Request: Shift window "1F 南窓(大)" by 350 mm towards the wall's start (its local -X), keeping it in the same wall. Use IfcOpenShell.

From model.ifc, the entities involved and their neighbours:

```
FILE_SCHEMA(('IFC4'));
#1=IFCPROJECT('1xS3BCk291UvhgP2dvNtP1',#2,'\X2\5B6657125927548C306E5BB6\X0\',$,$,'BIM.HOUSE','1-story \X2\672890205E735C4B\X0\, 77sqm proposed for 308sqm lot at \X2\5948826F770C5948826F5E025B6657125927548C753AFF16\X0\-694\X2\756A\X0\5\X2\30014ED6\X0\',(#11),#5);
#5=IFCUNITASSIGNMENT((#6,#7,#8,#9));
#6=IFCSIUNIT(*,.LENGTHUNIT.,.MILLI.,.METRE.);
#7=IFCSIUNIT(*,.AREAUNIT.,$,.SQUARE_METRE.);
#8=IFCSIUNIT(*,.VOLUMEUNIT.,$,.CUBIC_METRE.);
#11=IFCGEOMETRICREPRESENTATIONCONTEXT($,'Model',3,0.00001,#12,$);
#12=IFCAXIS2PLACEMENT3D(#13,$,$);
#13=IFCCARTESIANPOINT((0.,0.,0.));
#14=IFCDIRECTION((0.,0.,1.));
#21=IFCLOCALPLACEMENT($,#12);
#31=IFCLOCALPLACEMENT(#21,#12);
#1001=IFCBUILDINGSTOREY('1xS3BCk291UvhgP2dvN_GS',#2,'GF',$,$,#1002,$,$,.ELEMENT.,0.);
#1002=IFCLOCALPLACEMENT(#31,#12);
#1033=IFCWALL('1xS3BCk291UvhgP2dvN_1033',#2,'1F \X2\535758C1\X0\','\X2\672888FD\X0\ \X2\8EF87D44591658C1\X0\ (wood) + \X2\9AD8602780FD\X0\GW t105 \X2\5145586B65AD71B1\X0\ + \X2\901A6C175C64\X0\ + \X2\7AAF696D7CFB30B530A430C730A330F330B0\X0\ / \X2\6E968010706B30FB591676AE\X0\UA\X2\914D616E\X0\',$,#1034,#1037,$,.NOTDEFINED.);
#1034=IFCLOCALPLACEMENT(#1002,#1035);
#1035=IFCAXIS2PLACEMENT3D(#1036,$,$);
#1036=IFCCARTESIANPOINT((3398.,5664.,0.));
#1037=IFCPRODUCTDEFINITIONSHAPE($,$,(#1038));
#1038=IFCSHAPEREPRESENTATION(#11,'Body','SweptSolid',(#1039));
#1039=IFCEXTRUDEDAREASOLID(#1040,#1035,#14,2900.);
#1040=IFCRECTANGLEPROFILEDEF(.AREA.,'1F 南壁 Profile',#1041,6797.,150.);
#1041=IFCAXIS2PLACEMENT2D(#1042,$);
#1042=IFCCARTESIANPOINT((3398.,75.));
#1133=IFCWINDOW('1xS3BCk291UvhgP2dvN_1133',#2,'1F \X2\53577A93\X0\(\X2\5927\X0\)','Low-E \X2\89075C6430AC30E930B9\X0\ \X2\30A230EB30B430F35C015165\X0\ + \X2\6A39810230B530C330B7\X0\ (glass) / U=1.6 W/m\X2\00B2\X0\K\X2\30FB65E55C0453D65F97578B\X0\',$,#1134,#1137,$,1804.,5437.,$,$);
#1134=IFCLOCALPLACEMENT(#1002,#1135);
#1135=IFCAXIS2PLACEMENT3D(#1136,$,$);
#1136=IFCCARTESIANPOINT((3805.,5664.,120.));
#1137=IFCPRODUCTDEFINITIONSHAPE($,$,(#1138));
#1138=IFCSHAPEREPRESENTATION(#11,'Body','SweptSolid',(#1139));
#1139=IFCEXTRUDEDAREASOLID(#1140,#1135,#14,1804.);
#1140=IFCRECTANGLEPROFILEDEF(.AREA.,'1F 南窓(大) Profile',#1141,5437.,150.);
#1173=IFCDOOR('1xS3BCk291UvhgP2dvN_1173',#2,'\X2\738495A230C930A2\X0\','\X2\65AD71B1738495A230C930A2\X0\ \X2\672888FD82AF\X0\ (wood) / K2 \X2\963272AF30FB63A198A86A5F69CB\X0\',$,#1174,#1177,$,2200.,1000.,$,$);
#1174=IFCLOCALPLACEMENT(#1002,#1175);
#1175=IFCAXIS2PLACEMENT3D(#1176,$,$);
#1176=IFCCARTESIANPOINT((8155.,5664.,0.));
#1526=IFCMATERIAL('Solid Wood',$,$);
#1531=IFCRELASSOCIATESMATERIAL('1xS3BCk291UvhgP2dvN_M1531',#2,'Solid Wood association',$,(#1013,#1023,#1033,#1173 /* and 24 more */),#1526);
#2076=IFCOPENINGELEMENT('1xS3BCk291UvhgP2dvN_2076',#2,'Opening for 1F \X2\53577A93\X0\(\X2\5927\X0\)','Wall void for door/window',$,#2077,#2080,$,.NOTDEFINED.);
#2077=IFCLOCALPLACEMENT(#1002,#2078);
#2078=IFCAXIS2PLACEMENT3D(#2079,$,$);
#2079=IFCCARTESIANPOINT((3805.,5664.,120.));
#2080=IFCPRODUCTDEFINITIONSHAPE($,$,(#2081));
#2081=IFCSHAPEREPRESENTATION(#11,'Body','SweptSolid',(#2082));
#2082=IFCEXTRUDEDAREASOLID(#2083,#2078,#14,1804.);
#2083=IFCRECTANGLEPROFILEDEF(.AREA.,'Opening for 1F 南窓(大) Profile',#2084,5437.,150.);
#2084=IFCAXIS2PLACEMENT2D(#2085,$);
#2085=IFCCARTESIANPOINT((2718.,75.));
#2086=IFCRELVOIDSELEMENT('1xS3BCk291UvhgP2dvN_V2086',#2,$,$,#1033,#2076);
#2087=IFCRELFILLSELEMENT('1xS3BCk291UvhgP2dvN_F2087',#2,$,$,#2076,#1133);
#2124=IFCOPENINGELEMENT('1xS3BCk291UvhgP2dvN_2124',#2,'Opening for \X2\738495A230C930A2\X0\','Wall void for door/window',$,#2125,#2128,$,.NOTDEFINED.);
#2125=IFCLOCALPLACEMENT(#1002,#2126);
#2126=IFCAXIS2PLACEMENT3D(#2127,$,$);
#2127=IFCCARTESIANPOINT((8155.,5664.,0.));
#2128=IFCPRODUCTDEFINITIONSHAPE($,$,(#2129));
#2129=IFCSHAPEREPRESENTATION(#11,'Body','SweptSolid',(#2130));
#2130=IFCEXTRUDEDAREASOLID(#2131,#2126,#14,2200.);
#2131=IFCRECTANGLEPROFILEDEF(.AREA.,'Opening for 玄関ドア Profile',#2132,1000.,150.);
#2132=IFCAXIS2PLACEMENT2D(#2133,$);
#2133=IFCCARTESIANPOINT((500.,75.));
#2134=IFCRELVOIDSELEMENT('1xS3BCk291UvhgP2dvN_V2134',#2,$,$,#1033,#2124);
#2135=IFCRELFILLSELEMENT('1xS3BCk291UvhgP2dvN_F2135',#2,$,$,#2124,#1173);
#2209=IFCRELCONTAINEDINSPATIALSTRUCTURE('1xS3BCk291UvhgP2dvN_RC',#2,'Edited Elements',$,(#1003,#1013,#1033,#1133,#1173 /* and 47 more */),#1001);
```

```python
import ifcopenshell
import ifcopenshell.api.geometry
import ifcopenshell.util.placement

model = ifcopenshell.open("model.ifc")

window = model.by_guid("1xS3BCk291UvhgP2dvN_1133")
opening = window.FillsVoids[0].RelatingOpeningElement
wall = opening.VoidsElements[0].RelatingBuildingElement

wall_matrix = ifcopenshell.util.placement.get_local_placement(wall.ObjectPlacement)
shift = wall_matrix[:3, 0] * -350.0
before = ifcopenshell.util.placement.get_local_placement(window.ObjectPlacement)[:3, 3].copy()

# The window is not placed relative to its opening, so move both.
for product in (opening, window):
    matrix = ifcopenshell.util.placement.get_local_placement(product.ObjectPlacement)
    matrix[:3, 3] += shift
    ifcopenshell.api.geometry.edit_object_placement(model, product=product, matrix=matrix, is_si=False)

after = ifcopenshell.util.placement.get_local_placement(window.ObjectPlacement)[:3, 3]
print("window moved by", (after - before).round(3) + 0.0)

model.write("model_rev.ifc")
```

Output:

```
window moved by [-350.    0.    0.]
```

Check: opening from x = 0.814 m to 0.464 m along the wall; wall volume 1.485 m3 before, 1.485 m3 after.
